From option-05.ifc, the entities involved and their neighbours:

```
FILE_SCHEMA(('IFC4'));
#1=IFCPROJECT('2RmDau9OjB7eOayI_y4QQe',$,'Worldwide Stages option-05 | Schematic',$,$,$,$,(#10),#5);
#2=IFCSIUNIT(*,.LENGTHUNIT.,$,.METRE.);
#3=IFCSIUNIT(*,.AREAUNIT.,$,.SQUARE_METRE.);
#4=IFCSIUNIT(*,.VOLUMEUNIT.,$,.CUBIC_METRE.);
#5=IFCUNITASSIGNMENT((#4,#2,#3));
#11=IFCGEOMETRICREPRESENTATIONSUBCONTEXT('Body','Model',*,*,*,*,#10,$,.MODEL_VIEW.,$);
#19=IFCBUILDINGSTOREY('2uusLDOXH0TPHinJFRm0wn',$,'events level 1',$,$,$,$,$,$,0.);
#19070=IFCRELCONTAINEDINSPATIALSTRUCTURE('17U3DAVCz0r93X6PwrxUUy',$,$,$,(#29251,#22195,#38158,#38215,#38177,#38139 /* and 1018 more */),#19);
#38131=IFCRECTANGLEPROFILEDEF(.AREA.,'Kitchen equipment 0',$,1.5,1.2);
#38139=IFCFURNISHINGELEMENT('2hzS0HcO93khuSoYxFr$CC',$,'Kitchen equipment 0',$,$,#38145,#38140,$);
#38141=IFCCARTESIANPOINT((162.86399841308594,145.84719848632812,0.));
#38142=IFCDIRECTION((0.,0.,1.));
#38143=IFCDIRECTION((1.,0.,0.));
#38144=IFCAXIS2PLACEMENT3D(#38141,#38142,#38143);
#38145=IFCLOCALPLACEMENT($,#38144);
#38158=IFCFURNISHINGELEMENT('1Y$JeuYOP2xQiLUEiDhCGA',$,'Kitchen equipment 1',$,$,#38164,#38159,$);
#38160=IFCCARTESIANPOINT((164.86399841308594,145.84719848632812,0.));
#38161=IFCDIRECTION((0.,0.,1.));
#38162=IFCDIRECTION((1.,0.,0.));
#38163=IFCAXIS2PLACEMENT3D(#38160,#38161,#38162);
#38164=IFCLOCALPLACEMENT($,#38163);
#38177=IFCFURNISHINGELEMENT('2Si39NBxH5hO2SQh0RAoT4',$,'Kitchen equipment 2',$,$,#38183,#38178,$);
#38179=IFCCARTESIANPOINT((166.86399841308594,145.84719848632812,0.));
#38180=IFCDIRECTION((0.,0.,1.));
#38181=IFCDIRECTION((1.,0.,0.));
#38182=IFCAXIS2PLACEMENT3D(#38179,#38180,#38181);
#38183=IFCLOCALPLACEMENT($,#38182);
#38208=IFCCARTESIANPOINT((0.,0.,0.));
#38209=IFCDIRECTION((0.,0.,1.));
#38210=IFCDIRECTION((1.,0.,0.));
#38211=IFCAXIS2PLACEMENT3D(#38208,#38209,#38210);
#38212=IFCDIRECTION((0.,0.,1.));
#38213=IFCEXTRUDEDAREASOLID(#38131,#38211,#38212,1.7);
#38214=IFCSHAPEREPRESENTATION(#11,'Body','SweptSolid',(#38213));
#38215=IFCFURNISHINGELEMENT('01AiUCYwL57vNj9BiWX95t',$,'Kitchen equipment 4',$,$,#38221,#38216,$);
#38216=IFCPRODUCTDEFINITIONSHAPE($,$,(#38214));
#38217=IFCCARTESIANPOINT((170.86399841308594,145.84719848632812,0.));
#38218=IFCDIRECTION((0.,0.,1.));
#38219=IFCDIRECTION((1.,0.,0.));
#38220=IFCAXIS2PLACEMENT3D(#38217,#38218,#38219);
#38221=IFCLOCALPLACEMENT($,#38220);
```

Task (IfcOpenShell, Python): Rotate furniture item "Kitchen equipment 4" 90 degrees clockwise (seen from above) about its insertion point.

```python
import ifcopenshell
import ifcopenshell.api.geometry
import ifcopenshell.util.placement

model = ifcopenshell.open("option-05.ifc")

item = model.by_guid("01AiUCYwL57vNj9BiWX95t")
matrix = ifcopenshell.util.placement.get_local_placement(item.ObjectPlacement)
matrix = matrix @ ifcopenshell.util.placement.rotation(-90, "Z")
ifcopenshell.api.geometry.edit_object_placement(model, product=item, matrix=matrix, is_si=False)

print(ifcopenshell.util.placement.get_local_placement(item.ObjectPlacement).round(3) + 0.0)

model.write("option-05_v2.ifc")
```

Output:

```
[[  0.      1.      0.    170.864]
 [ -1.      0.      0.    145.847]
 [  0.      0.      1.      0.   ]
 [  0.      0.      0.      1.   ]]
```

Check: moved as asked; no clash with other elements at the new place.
